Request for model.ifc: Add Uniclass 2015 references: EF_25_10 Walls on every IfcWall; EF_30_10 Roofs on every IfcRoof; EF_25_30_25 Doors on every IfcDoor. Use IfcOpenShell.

First a look at what the model holds.

```python
import ifcopenshell

model = ifcopenshell.open("model.ifc")
print(model.schema)
print("classifications:", [c.Name for c in model.by_type("IfcClassification")])
for ifc_class in ("IfcDoor", "IfcRoof", "IfcStair", "IfcWall", "IfcWindow"):
    print(ifc_class, len(model.by_type(ifc_class)))
```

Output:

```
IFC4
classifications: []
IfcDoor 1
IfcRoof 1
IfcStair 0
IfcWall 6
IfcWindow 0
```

```python
import ifcopenshell
import ifcopenshell.api.classification

model = ifcopenshell.open("model.ifc")

system = ifcopenshell.api.classification.add_classification(model, classification="Uniclass 2015")

codes = {
    "IfcWall": ("EF_25_10", "Walls"),
    "IfcRoof": ("EF_30_10", "Roofs"),
    "IfcDoor": ("EF_25_30_25", "Doors"),
}
for ifc_class, (code, name) in codes.items():
    products = model.by_type(ifc_class)
    ifcopenshell.api.classification.add_reference(
        model, products=products, classification=system, identification=code, name=name
    )
    print(code, len(products))

model.write("model_edited.ifc")
```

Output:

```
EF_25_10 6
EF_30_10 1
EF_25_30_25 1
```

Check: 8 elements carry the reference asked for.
